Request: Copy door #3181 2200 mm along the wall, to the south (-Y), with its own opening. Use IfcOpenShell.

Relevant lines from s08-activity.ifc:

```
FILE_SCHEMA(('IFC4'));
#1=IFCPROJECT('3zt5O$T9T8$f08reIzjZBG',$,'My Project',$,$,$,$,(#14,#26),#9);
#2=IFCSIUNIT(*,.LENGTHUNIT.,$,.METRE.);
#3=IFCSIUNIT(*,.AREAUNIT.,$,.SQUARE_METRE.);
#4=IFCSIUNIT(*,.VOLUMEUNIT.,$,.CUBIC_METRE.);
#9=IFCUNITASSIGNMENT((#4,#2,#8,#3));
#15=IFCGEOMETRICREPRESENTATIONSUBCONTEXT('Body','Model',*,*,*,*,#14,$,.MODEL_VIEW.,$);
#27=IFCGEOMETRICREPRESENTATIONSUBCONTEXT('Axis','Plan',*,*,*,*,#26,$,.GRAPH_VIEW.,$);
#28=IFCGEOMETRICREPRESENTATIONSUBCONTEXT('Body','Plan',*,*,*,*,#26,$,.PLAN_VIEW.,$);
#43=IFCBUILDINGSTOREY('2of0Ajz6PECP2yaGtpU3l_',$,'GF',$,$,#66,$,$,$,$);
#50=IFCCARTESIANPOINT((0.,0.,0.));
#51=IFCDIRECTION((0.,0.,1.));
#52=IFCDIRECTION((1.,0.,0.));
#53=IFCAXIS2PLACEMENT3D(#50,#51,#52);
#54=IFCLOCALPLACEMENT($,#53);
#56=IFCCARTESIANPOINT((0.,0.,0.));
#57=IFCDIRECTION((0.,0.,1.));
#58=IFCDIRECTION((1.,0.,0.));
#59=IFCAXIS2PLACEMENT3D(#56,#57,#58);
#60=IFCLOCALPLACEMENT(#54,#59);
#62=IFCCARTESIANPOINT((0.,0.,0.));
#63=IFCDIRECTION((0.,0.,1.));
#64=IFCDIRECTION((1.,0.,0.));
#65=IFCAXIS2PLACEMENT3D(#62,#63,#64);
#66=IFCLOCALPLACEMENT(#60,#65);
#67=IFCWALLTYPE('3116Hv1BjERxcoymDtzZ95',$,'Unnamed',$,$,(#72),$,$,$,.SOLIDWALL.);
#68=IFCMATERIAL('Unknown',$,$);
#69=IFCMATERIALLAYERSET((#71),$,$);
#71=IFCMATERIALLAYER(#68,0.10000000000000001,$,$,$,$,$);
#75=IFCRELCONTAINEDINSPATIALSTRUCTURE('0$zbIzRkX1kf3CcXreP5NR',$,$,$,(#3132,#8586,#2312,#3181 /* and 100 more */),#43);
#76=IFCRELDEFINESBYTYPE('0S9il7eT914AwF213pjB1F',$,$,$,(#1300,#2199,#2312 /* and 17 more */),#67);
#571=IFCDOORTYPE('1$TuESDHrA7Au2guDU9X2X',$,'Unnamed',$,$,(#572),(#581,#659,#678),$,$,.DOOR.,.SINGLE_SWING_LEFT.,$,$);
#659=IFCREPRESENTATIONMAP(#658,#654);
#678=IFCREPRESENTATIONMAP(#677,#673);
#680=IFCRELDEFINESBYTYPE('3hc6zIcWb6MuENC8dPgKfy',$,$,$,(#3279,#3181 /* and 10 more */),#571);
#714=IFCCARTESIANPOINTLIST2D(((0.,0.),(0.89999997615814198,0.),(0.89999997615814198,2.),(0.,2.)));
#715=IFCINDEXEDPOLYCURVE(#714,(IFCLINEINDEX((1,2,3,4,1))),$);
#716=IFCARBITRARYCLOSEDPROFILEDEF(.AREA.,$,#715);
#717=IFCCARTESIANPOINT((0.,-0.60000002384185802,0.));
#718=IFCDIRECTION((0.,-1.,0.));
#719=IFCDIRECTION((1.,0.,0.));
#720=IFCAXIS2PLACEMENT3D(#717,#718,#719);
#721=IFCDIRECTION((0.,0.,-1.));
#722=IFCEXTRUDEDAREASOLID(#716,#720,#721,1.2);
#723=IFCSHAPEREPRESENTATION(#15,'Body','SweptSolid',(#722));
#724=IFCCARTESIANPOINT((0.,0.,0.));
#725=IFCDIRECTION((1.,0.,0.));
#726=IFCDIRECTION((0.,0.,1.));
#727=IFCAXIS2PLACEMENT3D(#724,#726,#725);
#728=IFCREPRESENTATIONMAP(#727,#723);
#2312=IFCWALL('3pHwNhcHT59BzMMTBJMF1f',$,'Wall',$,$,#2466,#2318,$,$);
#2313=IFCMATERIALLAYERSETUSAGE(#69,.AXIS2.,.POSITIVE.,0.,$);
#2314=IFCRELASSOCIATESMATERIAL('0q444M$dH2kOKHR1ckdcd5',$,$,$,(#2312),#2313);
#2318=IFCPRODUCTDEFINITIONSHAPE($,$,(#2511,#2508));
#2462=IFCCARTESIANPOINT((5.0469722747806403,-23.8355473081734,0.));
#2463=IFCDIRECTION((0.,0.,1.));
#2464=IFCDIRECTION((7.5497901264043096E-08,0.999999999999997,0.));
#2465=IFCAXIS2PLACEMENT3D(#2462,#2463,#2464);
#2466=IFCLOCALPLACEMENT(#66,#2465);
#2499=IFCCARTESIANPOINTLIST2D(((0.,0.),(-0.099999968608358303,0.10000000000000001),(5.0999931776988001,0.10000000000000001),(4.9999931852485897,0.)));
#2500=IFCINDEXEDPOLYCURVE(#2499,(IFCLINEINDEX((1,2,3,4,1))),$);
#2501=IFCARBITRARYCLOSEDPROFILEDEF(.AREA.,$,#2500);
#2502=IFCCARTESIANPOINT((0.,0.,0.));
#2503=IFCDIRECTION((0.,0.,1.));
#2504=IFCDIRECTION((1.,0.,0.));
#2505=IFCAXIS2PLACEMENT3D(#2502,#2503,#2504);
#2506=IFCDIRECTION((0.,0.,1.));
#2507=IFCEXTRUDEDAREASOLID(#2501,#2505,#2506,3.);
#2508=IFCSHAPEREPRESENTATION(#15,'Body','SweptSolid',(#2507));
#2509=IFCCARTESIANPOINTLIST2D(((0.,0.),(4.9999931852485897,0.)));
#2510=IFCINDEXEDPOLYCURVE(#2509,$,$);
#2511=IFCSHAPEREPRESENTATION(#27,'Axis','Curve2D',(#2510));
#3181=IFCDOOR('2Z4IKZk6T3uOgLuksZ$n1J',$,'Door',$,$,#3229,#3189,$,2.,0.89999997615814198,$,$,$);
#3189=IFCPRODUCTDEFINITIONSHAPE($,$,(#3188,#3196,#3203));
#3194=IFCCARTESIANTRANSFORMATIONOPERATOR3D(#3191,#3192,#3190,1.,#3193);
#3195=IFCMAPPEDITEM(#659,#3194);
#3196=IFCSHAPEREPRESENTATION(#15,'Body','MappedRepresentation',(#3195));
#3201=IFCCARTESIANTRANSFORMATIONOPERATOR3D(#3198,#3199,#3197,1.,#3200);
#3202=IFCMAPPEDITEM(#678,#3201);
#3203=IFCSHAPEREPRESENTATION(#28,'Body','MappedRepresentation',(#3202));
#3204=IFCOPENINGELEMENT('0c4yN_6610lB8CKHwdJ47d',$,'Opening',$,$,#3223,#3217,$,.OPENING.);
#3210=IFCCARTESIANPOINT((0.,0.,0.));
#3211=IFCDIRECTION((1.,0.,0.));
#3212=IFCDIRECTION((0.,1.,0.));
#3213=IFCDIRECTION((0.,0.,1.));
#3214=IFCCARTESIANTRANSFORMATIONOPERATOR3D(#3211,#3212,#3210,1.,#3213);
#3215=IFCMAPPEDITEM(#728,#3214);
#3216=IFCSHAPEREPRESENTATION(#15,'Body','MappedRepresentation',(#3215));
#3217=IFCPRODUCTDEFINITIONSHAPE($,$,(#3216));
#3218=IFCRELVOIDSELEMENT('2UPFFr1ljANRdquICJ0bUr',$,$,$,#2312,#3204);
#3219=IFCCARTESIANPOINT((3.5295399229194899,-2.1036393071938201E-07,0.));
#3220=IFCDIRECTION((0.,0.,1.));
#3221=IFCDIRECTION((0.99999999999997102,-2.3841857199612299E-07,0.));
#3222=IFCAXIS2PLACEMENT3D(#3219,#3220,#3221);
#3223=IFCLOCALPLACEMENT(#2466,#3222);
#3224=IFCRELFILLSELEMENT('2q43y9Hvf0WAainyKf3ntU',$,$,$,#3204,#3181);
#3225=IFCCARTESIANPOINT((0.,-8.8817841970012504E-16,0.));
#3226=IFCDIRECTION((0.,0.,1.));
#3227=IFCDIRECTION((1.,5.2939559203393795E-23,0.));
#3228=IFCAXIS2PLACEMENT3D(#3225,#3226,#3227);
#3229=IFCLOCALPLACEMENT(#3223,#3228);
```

```python
import ifcopenshell
import ifcopenshell.api.feature
import ifcopenshell.api.geometry
import ifcopenshell.api.root
import ifcopenshell.geom
import ifcopenshell.util.element
import ifcopenshell.util.placement
import ifcopenshell.util.shape
import ifcopenshell.util.unit

model = ifcopenshell.open("s08-activity.ifc")
unit_scale = ifcopenshell.util.unit.calculate_unit_scale(model)
settings = ifcopenshell.geom.settings()


def volume(element):
    """Net volume in cubic metres, openings subtracted."""
    shape = ifcopenshell.geom.create_shape(settings, element)
    return ifcopenshell.util.shape.get_volume(shape.geometry)


door = model.by_guid("2Z4IKZk6T3uOgLuksZ$n1J")
opening = door.FillsVoids[0].RelatingOpeningElement
wall = opening.VoidsElements[0].RelatingBuildingElement
before = volume(wall)
shift = ifcopenshell.util.placement.get_local_placement(wall.ObjectPlacement)[:3, 0] * -2.2 / unit_scale

# copy_class copies the void relationship, type, container and properties, but no geometry.
new_opening = ifcopenshell.api.root.copy_class(model, product=opening)
new_opening.Representation = ifcopenshell.util.element.copy_deep(
    model, opening.Representation, exclude=["IfcGeometricRepresentationContext", "IfcRepresentationMap"]
)
new_door = ifcopenshell.api.root.copy_class(model, product=door)
new_door.Representation = ifcopenshell.util.element.copy_deep(
    model, door.Representation, exclude=["IfcGeometricRepresentationContext", "IfcRepresentationMap"]
)
ifcopenshell.api.feature.add_filling(model, opening=new_opening, element=new_door)

for old, new in ((opening, new_opening), (door, new_door)):
    matrix = ifcopenshell.util.placement.get_local_placement(old.ObjectPlacement)
    matrix[:3, 3] += shift
    ifcopenshell.api.geometry.edit_object_placement(model, product=new, matrix=matrix, is_si=False)

after = volume(wall)

print(f"wall volume {before:.3f} -> {after:.3f} m3")

model.write("s08-activity_edited.ifc")
```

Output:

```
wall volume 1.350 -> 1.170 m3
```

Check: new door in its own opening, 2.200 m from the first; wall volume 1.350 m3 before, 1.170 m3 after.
